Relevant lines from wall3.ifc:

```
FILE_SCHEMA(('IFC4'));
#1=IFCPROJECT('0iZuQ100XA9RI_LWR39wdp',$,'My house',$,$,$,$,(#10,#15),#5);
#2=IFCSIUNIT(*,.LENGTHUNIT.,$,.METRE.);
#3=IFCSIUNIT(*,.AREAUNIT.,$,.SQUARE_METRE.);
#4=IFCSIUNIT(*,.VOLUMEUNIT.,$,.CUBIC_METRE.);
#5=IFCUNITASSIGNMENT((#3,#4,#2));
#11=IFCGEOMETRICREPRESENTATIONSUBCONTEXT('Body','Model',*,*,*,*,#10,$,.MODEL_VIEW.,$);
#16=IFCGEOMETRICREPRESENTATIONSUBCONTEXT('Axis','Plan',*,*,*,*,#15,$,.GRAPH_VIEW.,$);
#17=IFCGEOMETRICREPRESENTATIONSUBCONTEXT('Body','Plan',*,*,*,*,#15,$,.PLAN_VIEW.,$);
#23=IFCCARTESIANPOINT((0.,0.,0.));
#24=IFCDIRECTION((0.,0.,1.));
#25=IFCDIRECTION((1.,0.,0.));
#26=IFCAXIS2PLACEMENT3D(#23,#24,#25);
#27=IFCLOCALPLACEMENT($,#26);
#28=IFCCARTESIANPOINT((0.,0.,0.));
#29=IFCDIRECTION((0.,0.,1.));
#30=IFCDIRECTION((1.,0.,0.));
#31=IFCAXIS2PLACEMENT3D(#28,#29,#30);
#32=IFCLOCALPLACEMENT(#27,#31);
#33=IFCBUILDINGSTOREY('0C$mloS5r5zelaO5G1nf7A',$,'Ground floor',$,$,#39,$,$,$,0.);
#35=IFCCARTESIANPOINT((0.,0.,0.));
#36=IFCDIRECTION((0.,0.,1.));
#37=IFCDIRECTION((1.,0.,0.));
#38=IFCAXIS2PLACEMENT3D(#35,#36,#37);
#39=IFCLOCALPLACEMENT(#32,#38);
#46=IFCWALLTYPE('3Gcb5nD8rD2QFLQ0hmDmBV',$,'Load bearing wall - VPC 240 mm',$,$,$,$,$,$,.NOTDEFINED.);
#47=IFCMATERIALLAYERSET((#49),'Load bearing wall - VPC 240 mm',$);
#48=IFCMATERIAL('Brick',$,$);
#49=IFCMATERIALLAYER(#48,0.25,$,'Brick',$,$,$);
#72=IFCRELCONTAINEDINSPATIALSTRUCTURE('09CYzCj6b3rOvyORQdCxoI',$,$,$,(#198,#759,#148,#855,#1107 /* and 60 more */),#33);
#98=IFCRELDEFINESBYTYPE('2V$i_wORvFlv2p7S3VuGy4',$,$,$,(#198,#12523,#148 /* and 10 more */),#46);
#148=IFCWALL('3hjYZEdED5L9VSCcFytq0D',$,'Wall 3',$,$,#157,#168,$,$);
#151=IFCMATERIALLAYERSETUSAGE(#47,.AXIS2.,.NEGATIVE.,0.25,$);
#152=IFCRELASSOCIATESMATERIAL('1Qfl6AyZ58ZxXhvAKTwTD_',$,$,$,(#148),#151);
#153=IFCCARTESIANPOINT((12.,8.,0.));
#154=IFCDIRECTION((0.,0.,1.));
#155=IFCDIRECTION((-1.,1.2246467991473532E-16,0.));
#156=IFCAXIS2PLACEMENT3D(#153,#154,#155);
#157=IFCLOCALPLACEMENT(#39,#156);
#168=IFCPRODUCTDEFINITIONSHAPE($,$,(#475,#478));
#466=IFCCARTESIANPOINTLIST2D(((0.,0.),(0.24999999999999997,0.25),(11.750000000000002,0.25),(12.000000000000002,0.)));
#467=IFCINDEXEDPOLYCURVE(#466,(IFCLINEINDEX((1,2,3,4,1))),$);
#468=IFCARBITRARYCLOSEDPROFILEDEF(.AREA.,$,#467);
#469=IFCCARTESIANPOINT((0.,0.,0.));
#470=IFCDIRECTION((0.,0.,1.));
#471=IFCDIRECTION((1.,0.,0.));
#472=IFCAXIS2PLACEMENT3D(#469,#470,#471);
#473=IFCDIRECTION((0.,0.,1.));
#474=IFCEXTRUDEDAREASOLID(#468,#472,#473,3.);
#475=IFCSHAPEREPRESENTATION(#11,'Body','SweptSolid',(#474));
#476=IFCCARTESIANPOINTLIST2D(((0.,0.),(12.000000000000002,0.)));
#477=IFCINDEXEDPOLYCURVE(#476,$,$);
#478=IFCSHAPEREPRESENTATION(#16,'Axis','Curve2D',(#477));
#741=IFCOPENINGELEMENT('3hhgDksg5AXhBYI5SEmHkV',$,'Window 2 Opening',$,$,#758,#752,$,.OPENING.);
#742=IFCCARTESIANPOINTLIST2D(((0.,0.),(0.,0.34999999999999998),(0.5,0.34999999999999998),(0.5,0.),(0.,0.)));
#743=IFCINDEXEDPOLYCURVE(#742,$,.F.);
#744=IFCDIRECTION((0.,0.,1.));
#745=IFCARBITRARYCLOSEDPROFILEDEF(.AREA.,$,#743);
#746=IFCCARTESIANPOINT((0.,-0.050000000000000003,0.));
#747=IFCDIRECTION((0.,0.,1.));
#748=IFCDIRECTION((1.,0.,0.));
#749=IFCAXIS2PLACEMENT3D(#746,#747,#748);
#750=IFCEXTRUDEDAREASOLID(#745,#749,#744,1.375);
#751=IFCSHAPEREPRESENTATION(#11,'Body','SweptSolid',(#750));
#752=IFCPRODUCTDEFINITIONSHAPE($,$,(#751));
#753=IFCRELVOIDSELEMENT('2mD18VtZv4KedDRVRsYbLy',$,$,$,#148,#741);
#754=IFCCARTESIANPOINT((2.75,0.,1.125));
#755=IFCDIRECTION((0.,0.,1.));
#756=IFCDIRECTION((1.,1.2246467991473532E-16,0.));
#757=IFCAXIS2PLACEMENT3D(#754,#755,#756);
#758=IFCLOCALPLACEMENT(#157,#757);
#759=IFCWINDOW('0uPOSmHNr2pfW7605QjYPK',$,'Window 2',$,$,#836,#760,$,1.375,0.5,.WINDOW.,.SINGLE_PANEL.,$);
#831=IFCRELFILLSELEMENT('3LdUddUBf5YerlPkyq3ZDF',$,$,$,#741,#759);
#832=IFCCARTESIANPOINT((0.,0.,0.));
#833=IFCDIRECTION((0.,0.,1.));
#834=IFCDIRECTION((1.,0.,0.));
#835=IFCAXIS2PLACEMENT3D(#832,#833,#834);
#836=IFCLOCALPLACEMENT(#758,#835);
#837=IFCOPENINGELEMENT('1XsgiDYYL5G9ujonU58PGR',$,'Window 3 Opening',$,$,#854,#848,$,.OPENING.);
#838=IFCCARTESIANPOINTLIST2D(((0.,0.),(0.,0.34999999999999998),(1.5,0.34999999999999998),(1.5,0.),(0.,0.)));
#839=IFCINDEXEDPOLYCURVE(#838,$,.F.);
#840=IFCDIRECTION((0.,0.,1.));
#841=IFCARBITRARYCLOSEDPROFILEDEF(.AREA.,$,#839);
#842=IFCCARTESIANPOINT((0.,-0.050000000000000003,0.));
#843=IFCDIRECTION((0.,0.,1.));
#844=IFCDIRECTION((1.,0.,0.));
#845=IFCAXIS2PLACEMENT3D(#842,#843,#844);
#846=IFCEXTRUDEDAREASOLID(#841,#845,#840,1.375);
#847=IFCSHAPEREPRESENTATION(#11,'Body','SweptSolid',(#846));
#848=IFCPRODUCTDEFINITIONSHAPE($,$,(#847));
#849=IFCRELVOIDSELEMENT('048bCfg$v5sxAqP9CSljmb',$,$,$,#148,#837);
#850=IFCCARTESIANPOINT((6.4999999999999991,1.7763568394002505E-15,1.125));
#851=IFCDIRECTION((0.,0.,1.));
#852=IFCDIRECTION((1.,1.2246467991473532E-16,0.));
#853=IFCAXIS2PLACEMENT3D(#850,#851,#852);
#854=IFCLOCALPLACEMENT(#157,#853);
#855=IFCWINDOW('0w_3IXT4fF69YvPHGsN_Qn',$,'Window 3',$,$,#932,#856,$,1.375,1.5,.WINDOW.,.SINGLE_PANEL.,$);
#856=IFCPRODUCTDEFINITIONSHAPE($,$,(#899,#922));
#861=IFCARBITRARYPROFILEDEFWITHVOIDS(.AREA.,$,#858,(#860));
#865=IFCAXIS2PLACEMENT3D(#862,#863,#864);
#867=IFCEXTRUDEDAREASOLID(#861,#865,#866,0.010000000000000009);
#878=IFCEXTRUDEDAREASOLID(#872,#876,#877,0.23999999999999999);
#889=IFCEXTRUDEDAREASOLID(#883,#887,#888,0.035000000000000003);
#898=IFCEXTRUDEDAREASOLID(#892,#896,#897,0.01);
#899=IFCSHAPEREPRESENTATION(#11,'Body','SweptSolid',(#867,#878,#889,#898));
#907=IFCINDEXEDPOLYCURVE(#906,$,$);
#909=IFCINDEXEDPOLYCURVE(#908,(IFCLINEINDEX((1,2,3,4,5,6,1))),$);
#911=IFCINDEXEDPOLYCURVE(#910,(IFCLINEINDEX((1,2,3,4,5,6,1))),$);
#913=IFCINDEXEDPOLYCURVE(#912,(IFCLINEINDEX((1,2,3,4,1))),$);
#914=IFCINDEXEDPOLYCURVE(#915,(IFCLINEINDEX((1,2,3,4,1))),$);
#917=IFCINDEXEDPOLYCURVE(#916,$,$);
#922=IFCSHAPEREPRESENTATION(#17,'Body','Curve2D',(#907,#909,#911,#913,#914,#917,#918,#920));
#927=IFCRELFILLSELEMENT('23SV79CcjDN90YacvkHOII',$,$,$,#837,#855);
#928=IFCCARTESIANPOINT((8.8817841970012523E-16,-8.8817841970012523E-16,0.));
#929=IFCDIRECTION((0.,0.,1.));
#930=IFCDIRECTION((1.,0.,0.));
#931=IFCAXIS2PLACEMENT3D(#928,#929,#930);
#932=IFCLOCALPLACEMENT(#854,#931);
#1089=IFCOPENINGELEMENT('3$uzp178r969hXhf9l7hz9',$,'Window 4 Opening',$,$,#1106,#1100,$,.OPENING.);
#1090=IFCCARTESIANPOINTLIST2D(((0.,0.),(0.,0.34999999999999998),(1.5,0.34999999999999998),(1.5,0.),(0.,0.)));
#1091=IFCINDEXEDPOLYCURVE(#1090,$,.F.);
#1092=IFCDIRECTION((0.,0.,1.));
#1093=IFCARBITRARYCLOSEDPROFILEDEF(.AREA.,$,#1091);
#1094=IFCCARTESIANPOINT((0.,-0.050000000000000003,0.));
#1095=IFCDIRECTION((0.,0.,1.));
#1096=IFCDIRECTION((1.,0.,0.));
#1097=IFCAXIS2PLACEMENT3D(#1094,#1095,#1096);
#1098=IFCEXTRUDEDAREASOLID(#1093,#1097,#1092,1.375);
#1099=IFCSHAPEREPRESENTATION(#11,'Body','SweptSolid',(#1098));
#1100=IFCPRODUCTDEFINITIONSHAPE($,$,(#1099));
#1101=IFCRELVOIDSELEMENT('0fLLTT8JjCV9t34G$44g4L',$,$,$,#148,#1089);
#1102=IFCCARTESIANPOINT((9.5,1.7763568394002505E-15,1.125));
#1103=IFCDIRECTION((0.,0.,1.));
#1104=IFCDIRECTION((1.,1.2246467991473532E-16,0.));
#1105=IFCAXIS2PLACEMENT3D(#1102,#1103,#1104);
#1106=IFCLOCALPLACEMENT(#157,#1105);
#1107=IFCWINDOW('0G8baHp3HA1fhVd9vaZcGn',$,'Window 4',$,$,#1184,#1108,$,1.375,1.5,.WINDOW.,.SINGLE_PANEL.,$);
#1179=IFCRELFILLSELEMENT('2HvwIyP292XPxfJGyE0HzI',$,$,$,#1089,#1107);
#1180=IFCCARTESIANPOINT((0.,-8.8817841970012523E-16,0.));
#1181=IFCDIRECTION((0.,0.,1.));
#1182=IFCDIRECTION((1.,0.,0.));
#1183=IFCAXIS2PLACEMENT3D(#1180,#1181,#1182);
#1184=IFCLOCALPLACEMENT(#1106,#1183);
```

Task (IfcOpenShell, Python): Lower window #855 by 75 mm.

```python
import numpy as np
import ifcopenshell
import ifcopenshell.api.geometry
import ifcopenshell.util.placement
import ifcopenshell.util.unit

model = ifcopenshell.open("wall3.ifc")
unit_scale = ifcopenshell.util.unit.calculate_unit_scale(model)

window = model.by_id(855)
opening = window.FillsVoids[0].RelatingOpeningElement
dz = -0.075

shift = np.array([0.0, 0.0, dz])
# The window is placed relative to its opening, so it follows when the opening moves.
matrix = ifcopenshell.util.placement.get_local_placement(opening.ObjectPlacement)
matrix[:3, 3] += shift
ifcopenshell.api.geometry.edit_object_placement(
    model, product=opening, matrix=matrix, is_si=False, should_transform_children=True
)

print(f"moved by {dz * unit_scale:+.3f} m")

model.write("wall3_updated.ifc")
```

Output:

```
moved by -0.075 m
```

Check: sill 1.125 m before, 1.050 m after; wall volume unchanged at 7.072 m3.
